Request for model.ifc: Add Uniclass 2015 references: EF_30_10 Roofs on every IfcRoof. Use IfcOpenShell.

First a look at what the model holds.

```python
import ifcopenshell

model = ifcopenshell.open("model.ifc")
print(model.schema)
print("classifications:", [c.Name for c in model.by_type("IfcClassification")])
for ifc_class in ("IfcDoor", "IfcRoof", "IfcStair", "IfcWall", "IfcWindow"):
    print(ifc_class, len(model.by_type(ifc_class)))
```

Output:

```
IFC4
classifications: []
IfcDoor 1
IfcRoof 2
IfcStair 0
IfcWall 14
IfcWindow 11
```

```python
import ifcopenshell
import ifcopenshell.api.classification

model = ifcopenshell.open("model.ifc")

system = ifcopenshell.api.classification.add_classification(model, classification="Uniclass 2015")

codes = {
    "IfcRoof": ("EF_30_10", "Roofs"),
}
for ifc_class, (code, name) in codes.items():
    products = model.by_type(ifc_class)
    ifcopenshell.api.classification.add_reference(
        model, products=products, classification=system, identification=code, name=name
    )
    print(code, len(products))

model.write("model_rev.ifc")
```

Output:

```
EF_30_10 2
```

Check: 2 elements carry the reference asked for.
